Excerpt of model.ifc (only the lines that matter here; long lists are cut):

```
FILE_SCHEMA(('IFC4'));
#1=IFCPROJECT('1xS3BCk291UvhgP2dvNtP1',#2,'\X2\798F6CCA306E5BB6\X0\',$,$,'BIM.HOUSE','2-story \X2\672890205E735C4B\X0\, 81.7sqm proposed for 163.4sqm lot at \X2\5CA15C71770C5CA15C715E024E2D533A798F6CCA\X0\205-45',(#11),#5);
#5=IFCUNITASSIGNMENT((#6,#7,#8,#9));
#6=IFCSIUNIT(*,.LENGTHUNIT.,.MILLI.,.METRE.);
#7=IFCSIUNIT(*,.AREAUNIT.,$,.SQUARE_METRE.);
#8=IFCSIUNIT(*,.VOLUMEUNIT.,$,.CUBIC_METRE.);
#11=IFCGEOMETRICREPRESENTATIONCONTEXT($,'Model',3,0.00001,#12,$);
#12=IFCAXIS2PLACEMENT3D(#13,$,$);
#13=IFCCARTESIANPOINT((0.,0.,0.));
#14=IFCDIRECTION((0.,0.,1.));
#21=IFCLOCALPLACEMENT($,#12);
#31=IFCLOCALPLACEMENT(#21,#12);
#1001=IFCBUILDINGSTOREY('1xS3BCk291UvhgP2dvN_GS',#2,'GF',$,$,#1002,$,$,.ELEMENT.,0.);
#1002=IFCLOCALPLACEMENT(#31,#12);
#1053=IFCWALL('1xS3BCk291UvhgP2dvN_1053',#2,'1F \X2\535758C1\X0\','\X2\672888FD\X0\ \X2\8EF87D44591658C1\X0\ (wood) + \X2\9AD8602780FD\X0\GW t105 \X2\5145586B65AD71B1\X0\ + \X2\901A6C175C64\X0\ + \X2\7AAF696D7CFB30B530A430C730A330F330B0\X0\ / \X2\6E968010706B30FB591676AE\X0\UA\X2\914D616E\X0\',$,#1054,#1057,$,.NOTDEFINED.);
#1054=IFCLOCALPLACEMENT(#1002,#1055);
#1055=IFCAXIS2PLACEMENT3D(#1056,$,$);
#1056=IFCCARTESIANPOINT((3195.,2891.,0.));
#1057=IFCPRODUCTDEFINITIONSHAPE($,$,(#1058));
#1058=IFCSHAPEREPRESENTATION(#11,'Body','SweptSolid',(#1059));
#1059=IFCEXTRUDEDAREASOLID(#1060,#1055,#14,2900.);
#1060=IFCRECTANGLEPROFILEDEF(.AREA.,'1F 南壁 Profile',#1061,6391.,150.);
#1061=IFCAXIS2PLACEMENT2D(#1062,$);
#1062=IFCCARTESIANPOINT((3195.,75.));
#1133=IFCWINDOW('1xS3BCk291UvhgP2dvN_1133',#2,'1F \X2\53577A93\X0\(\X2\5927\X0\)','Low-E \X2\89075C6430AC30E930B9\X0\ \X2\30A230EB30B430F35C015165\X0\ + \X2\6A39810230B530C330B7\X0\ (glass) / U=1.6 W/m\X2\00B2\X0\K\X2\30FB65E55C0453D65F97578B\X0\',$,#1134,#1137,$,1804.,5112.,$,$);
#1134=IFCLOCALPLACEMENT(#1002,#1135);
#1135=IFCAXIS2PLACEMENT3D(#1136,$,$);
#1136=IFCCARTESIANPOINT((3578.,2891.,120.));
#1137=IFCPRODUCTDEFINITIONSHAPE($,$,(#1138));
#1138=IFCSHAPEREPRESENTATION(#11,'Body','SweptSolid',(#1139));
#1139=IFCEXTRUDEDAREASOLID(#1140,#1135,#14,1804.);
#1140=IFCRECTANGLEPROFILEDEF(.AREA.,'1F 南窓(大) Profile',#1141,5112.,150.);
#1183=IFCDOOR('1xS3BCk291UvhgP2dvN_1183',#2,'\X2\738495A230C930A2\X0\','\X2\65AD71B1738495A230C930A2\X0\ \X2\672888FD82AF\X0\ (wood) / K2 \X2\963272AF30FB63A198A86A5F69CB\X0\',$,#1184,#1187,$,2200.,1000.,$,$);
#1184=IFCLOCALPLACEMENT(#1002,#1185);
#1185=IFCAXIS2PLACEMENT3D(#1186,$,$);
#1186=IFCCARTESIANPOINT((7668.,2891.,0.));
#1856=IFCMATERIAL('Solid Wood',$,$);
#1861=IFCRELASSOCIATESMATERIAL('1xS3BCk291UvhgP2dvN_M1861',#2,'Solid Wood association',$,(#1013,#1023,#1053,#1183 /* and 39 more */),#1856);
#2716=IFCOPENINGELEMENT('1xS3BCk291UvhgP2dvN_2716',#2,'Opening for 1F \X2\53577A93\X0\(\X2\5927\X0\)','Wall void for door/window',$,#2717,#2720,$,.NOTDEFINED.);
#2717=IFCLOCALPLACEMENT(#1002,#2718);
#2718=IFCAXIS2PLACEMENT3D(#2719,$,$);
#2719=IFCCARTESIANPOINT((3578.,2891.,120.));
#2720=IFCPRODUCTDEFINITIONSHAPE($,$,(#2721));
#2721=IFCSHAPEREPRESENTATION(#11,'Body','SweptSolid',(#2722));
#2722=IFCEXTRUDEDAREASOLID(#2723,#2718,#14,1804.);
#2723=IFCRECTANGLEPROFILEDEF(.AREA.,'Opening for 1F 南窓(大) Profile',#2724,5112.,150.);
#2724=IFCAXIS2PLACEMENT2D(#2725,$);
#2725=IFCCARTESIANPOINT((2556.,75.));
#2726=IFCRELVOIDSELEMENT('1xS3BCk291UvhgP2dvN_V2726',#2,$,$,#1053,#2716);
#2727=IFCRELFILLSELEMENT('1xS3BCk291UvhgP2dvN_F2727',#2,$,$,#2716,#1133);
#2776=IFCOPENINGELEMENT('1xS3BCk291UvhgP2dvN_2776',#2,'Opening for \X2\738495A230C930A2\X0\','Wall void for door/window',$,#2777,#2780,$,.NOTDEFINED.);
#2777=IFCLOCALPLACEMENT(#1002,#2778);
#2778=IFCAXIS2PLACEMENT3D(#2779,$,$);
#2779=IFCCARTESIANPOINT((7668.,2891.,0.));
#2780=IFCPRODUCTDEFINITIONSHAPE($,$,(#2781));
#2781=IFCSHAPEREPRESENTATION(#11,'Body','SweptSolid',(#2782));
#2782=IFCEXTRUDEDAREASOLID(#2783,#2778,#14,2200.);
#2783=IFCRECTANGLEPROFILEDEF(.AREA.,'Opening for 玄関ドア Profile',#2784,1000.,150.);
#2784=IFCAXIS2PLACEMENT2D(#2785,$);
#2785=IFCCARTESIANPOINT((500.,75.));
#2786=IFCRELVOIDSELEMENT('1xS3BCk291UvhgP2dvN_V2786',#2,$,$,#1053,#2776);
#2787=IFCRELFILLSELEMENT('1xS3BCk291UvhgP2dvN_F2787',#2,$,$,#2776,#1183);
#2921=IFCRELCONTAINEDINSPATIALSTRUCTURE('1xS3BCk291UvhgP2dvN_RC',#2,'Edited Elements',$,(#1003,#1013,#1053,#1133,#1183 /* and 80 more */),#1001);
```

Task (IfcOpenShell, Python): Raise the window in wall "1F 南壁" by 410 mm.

```python
import numpy as np
import ifcopenshell
import ifcopenshell.api.geometry
import ifcopenshell.util.placement
import ifcopenshell.util.unit

model = ifcopenshell.open("model.ifc")
unit_scale = ifcopenshell.util.unit.calculate_unit_scale(model)

window = model.by_guid("1xS3BCk291UvhgP2dvN_1133")
opening = window.FillsVoids[0].RelatingOpeningElement
dz = 0.41 / unit_scale

shift = np.array([0.0, 0.0, dz])
# The window is not placed relative to its opening, so move both.
for product in (opening, window):
    matrix = ifcopenshell.util.placement.get_local_placement(product.ObjectPlacement)
    matrix[:3, 3] += shift
    ifcopenshell.api.geometry.edit_object_placement(model, product=product, matrix=matrix, is_si=False)

print(f"moved by {dz * unit_scale:+.3f} m")

model.write("model_edited.ifc")
```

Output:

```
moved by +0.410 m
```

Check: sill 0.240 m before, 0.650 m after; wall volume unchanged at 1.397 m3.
